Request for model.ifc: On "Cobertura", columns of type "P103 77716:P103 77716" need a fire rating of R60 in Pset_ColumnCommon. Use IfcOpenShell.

First a look at what the model holds.

```python
import ifcopenshell
import ifcopenshell.util.element

model = ifcopenshell.open("model.ifc")
print(model.schema)
storey = next(s for s in model.by_type("IfcBuildingStorey") if s.Name == "Cobertura")
columns = [e for e in ifcopenshell.util.element.get_decomposition(storey) if e.is_a("IfcColumn")]
seen = {}
for e in columns:
    element_type = ifcopenshell.util.element.get_type(e)
    key = (element_type.Name if element_type != e and element_type else None, ifcopenshell.util.element.get_pset(e, "Pset_ColumnCommon", "FireRating"))
    seen[key] = seen.get(key, 0) + 1
for (name, value), count in sorted(seen.items(), key=str):
    print(count, "x", name, "|", value)
```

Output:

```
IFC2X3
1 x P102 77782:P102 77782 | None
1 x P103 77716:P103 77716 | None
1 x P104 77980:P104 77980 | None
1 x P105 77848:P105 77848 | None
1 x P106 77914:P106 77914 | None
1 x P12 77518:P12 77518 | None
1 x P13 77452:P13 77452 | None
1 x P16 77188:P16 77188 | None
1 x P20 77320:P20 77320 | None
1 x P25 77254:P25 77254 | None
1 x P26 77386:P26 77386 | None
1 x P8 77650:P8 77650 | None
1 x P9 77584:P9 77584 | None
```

```python
import ifcopenshell
import ifcopenshell.api.pset
import ifcopenshell.util.element

model = ifcopenshell.open("model.ifc")

storey = next(s for s in model.by_type("IfcBuildingStorey") if s.Name == "Cobertura")
columns = [e for e in ifcopenshell.util.element.get_decomposition(storey) if e.is_a("IfcColumn")]

count = 0
for e in columns:
    element_type = ifcopenshell.util.element.get_type(e)
    if element_type in (None, e) or element_type.Name != "P103 77716:P103 77716":
        continue
    # add_pset returns the element's existing set when there is one.
    pset = ifcopenshell.api.pset.add_pset(model, product=e, name="Pset_ColumnCommon")
    ifcopenshell.api.pset.edit_pset(model, pset=pset, properties={"FireRating": "R60"})
    count += 1

print(count, "columns updated")

model.write("model-out.ifc")
```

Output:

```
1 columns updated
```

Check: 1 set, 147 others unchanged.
